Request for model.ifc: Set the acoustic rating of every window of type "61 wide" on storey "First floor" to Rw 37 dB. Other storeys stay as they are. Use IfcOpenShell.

First a look at what the model holds.

```python
import ifcopenshell
import ifcopenshell.util.element

model = ifcopenshell.open("model.ifc")
print(model.schema)
storey = next(s for s in model.by_type("IfcBuildingStorey") if s.Name == "First floor")
windows = [e for e in ifcopenshell.util.element.get_decomposition(storey) if e.is_a("IfcWindow")]
seen = {}
for e in windows:
    element_type = ifcopenshell.util.element.get_type(e)
    key = (element_type.Name if element_type != e and element_type else None, ifcopenshell.util.element.get_pset(e, "Pset_WindowCommon", "AcousticRating"))
    seen[key] = seen.get(key, 0) + 1
for (name, value), count in sorted(seen.items(), key=str):
    print(count, "x", name, "|", value)
```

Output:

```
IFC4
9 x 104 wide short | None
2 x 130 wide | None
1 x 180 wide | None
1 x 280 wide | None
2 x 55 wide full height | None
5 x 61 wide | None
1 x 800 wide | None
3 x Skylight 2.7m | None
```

```python
import ifcopenshell
import ifcopenshell.api.pset
import ifcopenshell.util.element

model = ifcopenshell.open("model.ifc")

storey = next(s for s in model.by_type("IfcBuildingStorey") if s.Name == "First floor")
windows = [e for e in ifcopenshell.util.element.get_decomposition(storey) if e.is_a("IfcWindow")]

count = 0
for e in windows:
    element_type = ifcopenshell.util.element.get_type(e)
    if element_type in (None, e) or element_type.Name != "61 wide":
        continue
    # add_pset returns the element's existing set when there is one.
    pset = ifcopenshell.api.pset.add_pset(model, product=e, name="Pset_WindowCommon")
    ifcopenshell.api.pset.edit_pset(model, pset=pset, properties={"AcousticRating": "Rw 37 dB"})
    count += 1

print(count, "windows updated")

model.write("model_rev.ifc")
```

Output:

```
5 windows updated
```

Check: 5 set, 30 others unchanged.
